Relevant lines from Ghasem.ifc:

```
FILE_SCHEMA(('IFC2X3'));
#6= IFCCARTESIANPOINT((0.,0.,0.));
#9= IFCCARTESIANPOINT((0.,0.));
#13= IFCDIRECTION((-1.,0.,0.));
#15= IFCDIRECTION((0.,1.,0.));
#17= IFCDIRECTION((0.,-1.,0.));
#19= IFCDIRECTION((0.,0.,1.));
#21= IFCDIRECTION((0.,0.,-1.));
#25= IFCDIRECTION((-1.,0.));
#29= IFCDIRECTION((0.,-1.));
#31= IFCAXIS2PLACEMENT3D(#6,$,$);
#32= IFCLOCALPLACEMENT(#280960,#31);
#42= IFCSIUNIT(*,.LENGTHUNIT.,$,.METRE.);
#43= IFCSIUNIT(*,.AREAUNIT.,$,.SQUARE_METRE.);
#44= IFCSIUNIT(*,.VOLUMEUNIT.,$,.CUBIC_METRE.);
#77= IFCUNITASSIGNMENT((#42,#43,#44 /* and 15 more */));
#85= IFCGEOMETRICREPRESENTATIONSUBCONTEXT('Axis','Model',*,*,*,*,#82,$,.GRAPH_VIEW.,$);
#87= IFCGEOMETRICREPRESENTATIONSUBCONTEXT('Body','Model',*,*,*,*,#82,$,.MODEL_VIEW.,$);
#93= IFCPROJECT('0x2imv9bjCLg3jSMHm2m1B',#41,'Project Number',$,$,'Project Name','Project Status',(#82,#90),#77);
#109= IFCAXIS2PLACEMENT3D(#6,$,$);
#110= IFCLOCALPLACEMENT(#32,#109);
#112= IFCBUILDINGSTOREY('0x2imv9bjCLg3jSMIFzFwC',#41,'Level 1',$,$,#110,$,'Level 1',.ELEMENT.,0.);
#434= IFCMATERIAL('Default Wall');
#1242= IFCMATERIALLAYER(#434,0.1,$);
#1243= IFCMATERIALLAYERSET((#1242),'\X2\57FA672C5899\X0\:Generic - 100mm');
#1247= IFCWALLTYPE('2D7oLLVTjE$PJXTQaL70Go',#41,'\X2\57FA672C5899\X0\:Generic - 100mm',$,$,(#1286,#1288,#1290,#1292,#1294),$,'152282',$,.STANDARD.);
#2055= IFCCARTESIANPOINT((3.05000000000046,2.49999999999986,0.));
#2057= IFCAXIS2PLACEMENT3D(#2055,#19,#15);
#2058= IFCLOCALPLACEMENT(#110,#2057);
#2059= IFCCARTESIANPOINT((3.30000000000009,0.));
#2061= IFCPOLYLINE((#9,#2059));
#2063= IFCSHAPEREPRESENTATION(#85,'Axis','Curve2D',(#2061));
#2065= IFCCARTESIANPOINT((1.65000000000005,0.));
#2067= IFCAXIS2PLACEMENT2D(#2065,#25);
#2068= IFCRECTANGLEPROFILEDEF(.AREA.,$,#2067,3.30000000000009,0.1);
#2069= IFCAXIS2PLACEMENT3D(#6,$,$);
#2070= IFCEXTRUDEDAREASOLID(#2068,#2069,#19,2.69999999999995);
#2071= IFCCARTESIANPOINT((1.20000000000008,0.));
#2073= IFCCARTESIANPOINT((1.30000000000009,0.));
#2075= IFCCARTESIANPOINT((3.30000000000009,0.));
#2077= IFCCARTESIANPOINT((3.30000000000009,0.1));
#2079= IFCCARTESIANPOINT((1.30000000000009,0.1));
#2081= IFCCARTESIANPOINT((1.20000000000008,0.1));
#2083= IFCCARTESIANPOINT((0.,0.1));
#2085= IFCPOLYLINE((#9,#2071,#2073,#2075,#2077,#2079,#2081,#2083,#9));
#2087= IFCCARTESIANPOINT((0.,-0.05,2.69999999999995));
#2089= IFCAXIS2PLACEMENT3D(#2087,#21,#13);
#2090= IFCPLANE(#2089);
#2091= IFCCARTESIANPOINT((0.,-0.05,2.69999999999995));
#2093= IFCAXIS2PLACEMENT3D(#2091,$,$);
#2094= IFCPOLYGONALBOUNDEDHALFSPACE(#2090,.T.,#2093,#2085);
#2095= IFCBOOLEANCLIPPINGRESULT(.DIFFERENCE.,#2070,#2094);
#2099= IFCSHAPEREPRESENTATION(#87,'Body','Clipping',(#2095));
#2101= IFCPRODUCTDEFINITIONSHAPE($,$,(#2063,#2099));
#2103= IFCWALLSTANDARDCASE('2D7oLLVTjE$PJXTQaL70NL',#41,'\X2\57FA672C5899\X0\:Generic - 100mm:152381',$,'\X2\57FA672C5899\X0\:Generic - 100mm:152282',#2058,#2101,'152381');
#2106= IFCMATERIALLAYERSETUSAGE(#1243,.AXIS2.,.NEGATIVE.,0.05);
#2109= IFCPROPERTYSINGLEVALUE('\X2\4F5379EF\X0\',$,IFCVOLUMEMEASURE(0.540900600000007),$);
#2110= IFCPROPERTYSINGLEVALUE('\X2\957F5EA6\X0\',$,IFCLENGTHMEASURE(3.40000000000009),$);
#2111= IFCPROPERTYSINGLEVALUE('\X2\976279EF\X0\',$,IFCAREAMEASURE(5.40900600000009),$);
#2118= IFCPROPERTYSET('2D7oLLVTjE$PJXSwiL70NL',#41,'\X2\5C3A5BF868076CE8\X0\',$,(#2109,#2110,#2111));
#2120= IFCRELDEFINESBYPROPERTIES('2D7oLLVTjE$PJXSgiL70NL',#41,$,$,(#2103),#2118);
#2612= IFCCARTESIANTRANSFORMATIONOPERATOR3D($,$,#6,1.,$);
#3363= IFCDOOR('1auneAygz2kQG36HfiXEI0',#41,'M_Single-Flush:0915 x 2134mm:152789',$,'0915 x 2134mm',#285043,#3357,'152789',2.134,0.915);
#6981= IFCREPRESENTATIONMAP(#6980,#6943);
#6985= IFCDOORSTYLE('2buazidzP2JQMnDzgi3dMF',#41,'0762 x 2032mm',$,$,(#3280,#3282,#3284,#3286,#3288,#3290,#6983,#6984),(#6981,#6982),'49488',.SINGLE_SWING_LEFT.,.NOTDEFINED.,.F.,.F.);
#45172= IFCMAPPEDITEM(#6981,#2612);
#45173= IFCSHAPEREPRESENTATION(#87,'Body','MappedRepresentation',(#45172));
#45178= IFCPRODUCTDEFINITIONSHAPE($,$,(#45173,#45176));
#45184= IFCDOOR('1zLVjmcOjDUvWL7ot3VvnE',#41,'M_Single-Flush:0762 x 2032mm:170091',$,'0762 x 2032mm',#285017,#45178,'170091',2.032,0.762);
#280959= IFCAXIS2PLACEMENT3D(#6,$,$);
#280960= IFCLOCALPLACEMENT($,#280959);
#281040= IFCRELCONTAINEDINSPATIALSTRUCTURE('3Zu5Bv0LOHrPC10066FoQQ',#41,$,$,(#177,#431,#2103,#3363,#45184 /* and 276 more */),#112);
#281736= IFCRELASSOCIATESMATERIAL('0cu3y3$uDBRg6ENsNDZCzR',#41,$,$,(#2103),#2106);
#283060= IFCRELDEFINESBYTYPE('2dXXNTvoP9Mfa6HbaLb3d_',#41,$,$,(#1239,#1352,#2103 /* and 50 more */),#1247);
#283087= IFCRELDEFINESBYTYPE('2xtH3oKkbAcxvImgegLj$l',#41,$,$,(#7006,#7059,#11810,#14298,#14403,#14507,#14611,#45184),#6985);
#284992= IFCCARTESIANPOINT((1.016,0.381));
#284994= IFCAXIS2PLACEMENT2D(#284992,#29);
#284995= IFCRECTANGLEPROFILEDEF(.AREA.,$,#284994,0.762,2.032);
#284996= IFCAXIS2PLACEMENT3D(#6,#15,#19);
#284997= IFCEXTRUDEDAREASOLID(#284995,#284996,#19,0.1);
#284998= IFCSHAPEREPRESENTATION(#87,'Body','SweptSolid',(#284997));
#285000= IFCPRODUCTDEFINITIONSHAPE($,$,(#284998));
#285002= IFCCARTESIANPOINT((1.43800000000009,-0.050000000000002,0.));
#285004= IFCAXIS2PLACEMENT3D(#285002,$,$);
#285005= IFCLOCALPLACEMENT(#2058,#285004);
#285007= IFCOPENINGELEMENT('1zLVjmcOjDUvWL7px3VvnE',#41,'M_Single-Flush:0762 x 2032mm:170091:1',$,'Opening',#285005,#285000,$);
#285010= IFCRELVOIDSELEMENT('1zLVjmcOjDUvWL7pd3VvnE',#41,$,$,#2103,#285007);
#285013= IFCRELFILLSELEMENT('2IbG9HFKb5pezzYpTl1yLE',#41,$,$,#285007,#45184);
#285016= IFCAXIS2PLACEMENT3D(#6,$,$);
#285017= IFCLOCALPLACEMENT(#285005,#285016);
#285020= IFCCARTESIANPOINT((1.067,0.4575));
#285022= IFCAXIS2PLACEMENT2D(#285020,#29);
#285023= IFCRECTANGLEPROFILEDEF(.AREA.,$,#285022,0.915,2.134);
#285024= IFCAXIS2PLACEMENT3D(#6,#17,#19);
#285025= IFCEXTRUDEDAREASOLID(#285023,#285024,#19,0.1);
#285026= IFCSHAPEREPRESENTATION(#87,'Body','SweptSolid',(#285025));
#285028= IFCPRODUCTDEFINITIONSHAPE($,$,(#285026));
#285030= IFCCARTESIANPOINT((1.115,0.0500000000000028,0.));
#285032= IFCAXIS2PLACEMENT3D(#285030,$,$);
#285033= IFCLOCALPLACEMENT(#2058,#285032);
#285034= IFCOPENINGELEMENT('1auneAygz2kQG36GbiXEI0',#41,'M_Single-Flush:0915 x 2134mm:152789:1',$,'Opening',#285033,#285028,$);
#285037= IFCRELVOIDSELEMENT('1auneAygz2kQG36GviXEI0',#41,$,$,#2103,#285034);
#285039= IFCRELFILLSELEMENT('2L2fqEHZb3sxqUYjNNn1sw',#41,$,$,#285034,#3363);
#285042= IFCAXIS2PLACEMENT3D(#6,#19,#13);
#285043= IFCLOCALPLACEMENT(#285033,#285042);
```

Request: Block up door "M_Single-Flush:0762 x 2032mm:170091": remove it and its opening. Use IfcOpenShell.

```python
import ifcopenshell
import ifcopenshell.api.feature
import ifcopenshell.api.pset
import ifcopenshell.api.root
import ifcopenshell.geom
import ifcopenshell.util.element
import ifcopenshell.util.shape
import ifcopenshell.util.unit

model = ifcopenshell.open("Ghasem.ifc")
area_scale = ifcopenshell.util.unit.calculate_unit_scale(model, "AREAUNIT")
volume_scale = ifcopenshell.util.unit.calculate_unit_scale(model, "VOLUMEUNIT")
settings = ifcopenshell.geom.settings()


def volume(element):
    """Net volume in cubic metres, openings subtracted."""
    shape = ifcopenshell.geom.create_shape(settings, element)
    return ifcopenshell.util.shape.get_volume(shape.geometry)


door = model.by_guid("1zLVjmcOjDUvWL7ot3VvnE")
opening = door.FillsVoids[0].RelatingOpeningElement
wall = opening.VoidsElements[0].RelatingBuildingElement
before = volume(wall)

ifcopenshell.api.root.remove_product(model, product=door)
ifcopenshell.api.feature.remove_feature(model, feature=opening)

after = volume(wall)
thickness = 0.1  # wall thickness in metres

# Update the wall's stored quantities.
pset = model.by_id(ifcopenshell.util.element.get_pset(wall, "尺寸标注", should_inherit=False)["id"])
ifcopenshell.api.pset.edit_pset(model, pset=pset, properties={
    "体积": model.create_entity("IfcVolumeMeasure", after / volume_scale),
    "面积": model.create_entity("IfcAreaMeasure", after / thickness / area_scale),
})

print(f"wall volume {before:.3f} -> {after:.3f} m3")

model.write("Ghasem_edited.ifc")
```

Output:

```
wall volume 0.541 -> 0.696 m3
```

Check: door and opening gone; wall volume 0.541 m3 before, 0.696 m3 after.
